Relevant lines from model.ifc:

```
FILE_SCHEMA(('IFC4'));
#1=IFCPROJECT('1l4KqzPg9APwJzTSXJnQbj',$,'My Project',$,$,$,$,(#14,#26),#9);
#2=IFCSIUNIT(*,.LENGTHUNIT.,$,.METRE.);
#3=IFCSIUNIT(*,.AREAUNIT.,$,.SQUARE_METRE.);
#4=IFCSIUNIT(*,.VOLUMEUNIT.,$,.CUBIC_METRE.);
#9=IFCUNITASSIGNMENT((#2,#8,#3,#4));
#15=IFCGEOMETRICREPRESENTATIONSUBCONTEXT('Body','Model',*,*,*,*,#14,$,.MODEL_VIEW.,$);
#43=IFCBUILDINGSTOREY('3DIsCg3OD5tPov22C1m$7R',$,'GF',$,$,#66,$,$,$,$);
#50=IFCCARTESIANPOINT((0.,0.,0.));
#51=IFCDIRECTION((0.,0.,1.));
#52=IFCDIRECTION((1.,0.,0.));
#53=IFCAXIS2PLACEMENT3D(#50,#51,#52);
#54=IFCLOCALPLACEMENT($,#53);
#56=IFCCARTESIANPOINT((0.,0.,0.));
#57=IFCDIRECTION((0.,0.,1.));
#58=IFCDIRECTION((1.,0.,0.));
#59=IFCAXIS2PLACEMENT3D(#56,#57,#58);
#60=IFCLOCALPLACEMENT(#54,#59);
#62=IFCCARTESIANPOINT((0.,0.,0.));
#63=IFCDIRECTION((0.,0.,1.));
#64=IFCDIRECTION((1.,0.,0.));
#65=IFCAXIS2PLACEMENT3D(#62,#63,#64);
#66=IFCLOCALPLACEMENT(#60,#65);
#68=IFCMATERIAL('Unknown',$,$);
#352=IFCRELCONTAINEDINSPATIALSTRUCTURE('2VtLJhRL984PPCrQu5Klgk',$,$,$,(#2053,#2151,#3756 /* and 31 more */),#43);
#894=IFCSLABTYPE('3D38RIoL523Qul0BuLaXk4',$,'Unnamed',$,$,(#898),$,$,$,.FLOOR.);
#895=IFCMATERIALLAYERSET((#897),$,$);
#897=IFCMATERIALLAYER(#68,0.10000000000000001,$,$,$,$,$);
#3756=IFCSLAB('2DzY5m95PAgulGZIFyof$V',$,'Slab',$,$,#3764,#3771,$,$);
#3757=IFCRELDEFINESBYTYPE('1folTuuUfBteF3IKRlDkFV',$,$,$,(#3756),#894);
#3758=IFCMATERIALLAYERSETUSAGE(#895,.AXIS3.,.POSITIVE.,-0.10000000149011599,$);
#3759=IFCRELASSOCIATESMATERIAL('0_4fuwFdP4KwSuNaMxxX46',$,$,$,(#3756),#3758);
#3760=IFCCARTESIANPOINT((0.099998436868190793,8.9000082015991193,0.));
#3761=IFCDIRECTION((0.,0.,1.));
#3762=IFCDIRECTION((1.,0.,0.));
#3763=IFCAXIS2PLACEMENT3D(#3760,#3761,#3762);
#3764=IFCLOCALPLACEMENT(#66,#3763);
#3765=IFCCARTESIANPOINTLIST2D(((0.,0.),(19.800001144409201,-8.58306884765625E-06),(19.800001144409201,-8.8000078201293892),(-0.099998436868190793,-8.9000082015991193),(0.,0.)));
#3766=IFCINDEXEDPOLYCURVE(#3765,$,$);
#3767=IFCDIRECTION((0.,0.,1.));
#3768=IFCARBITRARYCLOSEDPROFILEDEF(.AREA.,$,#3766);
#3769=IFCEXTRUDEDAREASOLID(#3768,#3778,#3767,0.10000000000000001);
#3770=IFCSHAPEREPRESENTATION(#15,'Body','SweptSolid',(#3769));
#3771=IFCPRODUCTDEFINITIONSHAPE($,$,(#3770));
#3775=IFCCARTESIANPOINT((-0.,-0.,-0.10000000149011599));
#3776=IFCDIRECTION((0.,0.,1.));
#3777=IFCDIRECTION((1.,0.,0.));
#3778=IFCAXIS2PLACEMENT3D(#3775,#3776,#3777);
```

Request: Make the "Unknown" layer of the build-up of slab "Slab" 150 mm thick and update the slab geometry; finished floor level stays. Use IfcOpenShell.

```python
import ifcopenshell
import ifcopenshell.util.element
import ifcopenshell.util.representation
import ifcopenshell.util.unit

model = ifcopenshell.open("model.ifc")
unit_scale = ifcopenshell.util.unit.calculate_unit_scale(model)

layer_set = model.by_id(895)
layer = next(l for l in layer_set.MaterialLayers if l.Material and l.Material.Name == "Unknown")
change = 0.15 / unit_scale - layer.LayerThickness
layer.LayerThickness += change

# Geometry does not follow the layer set by itself.
slabs = [e for e in ifcopenshell.util.element.get_elements_by_material(model, layer_set) if e.is_a("IfcSlab")]
for slab in sorted(slabs, key=lambda e: e.id()):
    body = ifcopenshell.util.representation.get_representation(slab, "Model", "Body")
    solid = body.Items[0]
    old_depth = solid.Depth
    solid.Depth += change
    # Extruded upwards: lower the start of the extrusion so the top stays.
    x, y, z = solid.Position.Location.Coordinates
    solid.Position.Location = model.createIfcCartesianPoint((x, y, z - change))
    print(slab.id(), f"{old_depth:g} -> {solid.Depth:g}")

# The layers are counted up from the underside, which has moved.
for usage in {ifcopenshell.util.element.get_material(slab) for slab in slabs}:
    usage.OffsetFromReferenceLine -= change

model.write("model_edited.ifc")
```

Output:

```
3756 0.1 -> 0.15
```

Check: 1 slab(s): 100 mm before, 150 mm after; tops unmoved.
